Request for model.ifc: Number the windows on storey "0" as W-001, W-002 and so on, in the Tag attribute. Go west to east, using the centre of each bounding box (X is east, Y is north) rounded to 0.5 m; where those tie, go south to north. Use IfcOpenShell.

First a look at what the model holds.

```python
import ifcopenshell
import ifcopenshell.util.element
import ifcopenshell.util.placement

model = ifcopenshell.open("model.ifc")
print(model.schema)
storey = next(s for s in model.by_type("IfcBuildingStorey") if s.Name == "0")
windows = [e for e in ifcopenshell.util.element.get_decomposition(storey) if e.is_a("IfcWindow")]
for e in sorted(windows, key=lambda e: e.id()):
    origin = ifcopenshell.util.placement.get_local_placement(e.ObjectPlacement)[:3, 3]
    print(e.id(), e.Tag, e.Name, origin.round(2) + 0.0, sep=" | ")
```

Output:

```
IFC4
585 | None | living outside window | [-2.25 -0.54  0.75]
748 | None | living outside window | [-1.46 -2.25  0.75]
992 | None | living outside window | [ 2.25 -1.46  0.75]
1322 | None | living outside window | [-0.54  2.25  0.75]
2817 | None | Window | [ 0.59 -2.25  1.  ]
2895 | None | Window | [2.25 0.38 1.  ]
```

```python
import ifcopenshell
import ifcopenshell.geom
import ifcopenshell.util.element
import ifcopenshell.util.shape

model = ifcopenshell.open("model.ifc")
settings = ifcopenshell.geom.settings()
settings.set("use-world-coords", True)


def centre(element):
    shape = ifcopenshell.geom.create_shape(settings, element)
    return ifcopenshell.util.shape.get_bbox_centroid(shape.geometry)


storey = next(s for s in model.by_type("IfcBuildingStorey") if s.Name == "0")
windows = [e for e in ifcopenshell.util.element.get_decomposition(storey) if e.is_a("IfcWindow")]

# Insertion points can sit at a corner or the storey origin, so sort by the geometry (in metres).
centres = {e: centre(e) for e in windows}
windows.sort(key=lambda e: (round(centres[e][0] / 0.5), centres[e][1]))

for i, e in enumerate(windows, start=1):
    number = f"W-0{i:02d}"
    e.Tag = number
    print(e.id(), number)

model.write("model_updated.ifc")
```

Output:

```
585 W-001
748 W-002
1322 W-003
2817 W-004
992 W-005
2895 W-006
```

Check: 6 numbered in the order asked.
